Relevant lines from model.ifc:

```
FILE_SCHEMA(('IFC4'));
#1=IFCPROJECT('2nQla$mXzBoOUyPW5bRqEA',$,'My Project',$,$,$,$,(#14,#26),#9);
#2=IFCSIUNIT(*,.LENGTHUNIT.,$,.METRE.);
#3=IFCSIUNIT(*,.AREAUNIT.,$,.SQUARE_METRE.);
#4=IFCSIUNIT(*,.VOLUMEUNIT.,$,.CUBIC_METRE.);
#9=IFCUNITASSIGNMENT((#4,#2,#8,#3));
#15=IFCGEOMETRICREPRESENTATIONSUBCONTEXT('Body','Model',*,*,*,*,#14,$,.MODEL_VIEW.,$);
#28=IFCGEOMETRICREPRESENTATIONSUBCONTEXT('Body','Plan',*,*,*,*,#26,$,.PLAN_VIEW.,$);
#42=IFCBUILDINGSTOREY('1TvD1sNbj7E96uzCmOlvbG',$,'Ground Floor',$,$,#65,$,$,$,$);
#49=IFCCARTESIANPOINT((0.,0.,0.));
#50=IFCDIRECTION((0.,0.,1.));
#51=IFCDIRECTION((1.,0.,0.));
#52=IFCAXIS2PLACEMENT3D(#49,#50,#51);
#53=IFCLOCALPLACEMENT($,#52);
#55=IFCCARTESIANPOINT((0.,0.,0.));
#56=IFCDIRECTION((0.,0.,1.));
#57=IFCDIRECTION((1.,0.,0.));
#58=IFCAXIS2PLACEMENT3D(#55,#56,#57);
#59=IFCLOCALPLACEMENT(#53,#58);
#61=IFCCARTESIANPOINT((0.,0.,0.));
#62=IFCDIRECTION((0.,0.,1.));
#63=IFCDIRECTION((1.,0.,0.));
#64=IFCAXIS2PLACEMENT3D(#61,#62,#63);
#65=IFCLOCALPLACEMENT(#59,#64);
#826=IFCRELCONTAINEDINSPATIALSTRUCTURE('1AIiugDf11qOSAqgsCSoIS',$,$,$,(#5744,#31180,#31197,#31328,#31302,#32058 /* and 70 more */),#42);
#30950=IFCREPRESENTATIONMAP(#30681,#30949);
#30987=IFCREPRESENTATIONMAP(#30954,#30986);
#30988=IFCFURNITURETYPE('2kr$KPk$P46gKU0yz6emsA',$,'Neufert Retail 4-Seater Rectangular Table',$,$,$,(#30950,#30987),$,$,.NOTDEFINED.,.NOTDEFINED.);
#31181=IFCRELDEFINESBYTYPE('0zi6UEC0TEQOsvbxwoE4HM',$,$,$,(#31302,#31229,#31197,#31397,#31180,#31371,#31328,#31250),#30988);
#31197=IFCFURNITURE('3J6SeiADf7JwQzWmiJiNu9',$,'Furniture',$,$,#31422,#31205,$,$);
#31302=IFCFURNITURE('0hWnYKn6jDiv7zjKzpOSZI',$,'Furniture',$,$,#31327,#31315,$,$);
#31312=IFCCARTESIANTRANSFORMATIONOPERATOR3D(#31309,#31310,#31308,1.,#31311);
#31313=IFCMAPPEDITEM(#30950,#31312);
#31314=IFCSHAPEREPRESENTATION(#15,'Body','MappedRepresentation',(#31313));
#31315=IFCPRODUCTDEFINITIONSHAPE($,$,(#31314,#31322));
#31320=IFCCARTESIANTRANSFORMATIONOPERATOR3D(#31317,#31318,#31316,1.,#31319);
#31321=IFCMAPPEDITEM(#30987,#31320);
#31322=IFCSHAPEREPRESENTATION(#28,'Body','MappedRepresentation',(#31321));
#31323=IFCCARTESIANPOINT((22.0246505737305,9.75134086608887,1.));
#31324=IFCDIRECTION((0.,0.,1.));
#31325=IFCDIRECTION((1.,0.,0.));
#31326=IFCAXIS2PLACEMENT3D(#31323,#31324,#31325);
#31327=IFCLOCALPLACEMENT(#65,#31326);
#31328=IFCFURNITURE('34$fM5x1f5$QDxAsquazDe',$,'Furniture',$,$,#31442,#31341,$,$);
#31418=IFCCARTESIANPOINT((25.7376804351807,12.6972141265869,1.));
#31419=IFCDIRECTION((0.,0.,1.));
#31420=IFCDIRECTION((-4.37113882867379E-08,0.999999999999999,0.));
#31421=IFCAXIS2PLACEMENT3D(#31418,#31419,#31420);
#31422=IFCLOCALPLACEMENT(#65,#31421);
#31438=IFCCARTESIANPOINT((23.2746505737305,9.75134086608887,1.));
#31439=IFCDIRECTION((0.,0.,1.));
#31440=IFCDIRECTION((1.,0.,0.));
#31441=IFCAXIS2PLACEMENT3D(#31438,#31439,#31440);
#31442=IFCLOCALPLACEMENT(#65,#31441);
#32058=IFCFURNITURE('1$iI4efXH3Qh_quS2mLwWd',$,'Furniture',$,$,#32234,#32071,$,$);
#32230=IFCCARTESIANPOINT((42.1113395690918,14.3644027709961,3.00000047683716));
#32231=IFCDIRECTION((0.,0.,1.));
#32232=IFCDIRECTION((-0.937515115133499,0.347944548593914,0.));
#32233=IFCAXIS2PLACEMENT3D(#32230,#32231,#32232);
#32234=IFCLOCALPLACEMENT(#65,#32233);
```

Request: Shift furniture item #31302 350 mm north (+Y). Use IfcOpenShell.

```python
import ifcopenshell
import ifcopenshell.api.geometry
import ifcopenshell.util.placement

model = ifcopenshell.open("model.ifc")

item = model.by_guid("0hWnYKn6jDiv7zjKzpOSZI")
matrix = ifcopenshell.util.placement.get_local_placement(item.ObjectPlacement)
matrix[1, 3] += 0.35
ifcopenshell.api.geometry.edit_object_placement(model, product=item, matrix=matrix, is_si=False)

print(ifcopenshell.util.placement.get_local_placement(item.ObjectPlacement).round(3) + 0.0)

model.write("model_edited.ifc")
```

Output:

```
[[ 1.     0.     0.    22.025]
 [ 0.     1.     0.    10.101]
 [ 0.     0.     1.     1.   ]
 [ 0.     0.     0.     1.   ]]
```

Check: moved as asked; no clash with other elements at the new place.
